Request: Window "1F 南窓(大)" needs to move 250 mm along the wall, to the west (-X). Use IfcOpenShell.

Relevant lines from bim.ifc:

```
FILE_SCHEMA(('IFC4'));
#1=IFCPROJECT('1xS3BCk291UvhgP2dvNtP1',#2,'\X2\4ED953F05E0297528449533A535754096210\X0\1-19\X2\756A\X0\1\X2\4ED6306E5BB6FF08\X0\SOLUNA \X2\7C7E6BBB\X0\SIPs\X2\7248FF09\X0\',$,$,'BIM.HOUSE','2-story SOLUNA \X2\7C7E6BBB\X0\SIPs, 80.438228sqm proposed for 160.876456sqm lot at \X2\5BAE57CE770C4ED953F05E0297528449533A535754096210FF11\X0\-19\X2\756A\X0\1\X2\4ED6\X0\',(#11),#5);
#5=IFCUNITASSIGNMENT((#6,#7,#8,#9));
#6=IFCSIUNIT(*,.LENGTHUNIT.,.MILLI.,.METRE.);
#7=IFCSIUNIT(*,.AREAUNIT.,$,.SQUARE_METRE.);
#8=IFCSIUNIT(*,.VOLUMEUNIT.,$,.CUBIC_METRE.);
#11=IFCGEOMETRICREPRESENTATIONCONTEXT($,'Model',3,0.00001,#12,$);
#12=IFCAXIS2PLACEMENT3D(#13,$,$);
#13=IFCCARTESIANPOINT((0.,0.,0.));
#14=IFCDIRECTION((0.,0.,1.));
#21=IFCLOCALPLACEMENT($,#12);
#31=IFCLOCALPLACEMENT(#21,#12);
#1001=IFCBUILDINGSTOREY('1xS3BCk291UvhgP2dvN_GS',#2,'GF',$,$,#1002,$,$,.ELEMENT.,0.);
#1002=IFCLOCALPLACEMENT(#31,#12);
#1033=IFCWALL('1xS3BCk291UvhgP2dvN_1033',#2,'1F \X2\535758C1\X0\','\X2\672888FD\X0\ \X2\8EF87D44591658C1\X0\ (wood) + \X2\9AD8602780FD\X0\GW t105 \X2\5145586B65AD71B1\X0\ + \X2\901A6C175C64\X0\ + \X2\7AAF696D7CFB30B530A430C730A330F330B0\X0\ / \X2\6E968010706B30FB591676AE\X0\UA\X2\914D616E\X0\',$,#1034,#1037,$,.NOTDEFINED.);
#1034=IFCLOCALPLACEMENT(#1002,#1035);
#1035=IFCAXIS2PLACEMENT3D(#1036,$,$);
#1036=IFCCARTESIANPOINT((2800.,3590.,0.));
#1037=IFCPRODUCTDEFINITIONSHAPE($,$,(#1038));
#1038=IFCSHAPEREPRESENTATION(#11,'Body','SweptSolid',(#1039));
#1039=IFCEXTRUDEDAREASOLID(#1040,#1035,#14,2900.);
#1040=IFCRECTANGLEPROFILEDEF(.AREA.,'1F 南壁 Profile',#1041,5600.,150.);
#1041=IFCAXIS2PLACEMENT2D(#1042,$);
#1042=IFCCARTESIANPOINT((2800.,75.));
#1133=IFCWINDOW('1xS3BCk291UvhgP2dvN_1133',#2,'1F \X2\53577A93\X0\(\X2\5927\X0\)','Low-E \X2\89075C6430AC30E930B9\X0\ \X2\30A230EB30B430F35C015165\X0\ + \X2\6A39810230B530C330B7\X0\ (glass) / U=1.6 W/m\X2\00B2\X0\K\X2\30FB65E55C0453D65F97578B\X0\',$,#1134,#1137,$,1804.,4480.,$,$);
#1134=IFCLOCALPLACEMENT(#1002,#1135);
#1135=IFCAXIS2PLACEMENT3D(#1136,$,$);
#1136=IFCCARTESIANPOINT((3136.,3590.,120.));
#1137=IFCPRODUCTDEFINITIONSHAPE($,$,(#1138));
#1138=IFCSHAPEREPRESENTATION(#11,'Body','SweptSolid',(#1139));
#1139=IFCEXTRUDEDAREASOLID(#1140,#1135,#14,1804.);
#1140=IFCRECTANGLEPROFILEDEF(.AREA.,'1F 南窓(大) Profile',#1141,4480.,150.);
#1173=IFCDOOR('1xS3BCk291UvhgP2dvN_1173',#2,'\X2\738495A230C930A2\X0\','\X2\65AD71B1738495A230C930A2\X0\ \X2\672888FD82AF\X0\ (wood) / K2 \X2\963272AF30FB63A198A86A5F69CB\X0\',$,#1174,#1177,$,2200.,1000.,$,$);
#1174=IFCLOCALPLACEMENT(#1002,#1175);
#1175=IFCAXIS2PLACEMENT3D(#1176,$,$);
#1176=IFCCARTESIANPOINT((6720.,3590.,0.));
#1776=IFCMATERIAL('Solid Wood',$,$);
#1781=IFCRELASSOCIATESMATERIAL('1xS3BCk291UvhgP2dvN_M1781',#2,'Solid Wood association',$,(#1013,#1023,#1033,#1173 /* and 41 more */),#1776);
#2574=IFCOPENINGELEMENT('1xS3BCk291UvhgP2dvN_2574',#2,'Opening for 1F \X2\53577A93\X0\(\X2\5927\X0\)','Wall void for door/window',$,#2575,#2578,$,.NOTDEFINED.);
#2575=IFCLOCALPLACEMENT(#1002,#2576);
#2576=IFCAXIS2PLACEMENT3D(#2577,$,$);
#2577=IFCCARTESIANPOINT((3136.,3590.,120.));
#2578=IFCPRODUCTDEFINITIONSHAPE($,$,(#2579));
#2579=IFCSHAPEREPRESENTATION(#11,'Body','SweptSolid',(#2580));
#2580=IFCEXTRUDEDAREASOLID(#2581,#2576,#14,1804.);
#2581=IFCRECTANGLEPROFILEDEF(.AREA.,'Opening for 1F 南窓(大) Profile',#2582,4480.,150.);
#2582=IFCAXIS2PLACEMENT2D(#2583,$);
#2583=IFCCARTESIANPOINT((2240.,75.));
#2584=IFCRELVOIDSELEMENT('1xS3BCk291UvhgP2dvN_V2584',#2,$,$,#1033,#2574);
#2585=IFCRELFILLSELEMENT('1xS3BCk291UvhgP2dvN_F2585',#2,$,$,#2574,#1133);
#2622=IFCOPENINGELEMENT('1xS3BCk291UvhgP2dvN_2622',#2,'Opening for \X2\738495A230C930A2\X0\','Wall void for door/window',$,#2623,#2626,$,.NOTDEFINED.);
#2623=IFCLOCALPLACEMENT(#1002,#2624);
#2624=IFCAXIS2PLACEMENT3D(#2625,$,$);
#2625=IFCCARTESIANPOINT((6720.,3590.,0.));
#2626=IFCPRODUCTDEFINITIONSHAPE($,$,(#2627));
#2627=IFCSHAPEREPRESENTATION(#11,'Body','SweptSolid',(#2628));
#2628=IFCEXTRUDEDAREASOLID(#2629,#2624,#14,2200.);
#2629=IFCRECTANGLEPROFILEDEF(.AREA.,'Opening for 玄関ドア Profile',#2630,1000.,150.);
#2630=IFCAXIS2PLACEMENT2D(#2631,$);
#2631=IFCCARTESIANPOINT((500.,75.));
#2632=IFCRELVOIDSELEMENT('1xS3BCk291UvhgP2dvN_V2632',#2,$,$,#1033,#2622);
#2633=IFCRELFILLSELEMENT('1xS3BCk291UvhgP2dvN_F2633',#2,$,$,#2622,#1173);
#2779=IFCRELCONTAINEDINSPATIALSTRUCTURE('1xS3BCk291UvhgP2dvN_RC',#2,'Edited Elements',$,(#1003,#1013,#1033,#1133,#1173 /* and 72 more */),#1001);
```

```python
import ifcopenshell
import ifcopenshell.api.geometry
import ifcopenshell.util.placement
import ifcopenshell.util.unit

model = ifcopenshell.open("bim.ifc")
unit_scale = ifcopenshell.util.unit.calculate_unit_scale(model)

window = model.by_id(1133)
opening = window.FillsVoids[0].RelatingOpeningElement
wall = opening.VoidsElements[0].RelatingBuildingElement

wall_matrix = ifcopenshell.util.placement.get_local_placement(wall.ObjectPlacement)
shift = wall_matrix[:3, 0] * -0.25 / unit_scale
before = ifcopenshell.util.placement.get_local_placement(window.ObjectPlacement)[:3, 3].copy()

# The window is not placed relative to its opening, so move both.
for product in (opening, window):
    matrix = ifcopenshell.util.placement.get_local_placement(product.ObjectPlacement)
    matrix[:3, 3] += shift
    ifcopenshell.api.geometry.edit_object_placement(model, product=product, matrix=matrix, is_si=False)

after = ifcopenshell.util.placement.get_local_placement(window.ObjectPlacement)[:3, 3]
print("window moved by", (after - before).round(3) + 0.0)

model.write("bim_updated.ifc")
```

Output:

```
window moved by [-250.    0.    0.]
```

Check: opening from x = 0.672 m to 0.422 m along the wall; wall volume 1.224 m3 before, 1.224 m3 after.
